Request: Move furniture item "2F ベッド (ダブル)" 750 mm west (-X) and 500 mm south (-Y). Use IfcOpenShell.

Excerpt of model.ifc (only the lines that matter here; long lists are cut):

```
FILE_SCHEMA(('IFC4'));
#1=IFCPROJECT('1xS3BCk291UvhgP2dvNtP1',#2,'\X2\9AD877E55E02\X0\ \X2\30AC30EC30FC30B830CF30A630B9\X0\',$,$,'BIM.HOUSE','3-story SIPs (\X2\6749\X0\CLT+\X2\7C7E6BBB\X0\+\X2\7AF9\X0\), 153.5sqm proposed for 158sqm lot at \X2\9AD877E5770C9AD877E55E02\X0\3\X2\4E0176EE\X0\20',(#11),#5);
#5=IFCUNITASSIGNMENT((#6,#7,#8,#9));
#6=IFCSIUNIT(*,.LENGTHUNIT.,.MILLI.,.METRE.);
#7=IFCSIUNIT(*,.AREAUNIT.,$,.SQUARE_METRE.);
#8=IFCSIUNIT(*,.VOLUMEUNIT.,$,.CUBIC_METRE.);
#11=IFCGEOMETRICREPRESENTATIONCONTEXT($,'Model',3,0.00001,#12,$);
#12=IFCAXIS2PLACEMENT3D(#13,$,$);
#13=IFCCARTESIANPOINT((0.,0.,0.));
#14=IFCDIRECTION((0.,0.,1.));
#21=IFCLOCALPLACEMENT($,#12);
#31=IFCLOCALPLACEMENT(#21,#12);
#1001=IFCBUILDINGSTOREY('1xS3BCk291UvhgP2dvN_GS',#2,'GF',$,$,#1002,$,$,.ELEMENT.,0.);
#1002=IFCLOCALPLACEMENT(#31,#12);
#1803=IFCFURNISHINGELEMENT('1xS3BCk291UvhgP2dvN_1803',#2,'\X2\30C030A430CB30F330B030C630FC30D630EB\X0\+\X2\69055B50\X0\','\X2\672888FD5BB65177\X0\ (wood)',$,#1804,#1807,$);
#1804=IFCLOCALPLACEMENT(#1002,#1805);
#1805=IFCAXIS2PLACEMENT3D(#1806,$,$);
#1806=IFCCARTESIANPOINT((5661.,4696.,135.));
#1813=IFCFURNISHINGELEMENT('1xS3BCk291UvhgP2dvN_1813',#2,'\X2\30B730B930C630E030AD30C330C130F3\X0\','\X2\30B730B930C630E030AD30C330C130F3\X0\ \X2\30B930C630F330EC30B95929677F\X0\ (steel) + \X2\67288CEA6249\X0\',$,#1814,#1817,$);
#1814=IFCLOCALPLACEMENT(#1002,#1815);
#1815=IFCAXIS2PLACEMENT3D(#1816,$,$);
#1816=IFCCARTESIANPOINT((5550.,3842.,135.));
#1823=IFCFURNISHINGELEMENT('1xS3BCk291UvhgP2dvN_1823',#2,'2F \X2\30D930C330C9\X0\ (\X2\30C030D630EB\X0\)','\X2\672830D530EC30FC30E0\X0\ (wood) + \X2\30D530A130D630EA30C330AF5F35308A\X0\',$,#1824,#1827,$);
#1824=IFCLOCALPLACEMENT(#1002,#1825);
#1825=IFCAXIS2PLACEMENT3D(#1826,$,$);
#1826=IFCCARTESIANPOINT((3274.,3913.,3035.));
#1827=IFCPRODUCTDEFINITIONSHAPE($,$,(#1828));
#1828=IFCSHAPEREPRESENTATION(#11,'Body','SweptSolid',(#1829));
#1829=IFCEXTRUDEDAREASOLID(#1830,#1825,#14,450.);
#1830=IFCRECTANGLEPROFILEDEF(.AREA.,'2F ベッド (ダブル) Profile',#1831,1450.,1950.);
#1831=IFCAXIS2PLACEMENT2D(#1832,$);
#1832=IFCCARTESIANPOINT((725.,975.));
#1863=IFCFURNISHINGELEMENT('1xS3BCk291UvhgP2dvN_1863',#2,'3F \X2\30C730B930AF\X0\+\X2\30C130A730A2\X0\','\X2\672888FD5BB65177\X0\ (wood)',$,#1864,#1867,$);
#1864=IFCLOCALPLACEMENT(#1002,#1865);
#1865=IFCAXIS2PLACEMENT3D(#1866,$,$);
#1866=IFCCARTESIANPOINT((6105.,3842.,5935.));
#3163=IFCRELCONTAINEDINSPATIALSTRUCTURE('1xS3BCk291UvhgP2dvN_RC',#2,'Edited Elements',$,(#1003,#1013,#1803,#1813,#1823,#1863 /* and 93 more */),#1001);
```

```python
import ifcopenshell
import ifcopenshell.api.geometry
import ifcopenshell.util.placement
import ifcopenshell.util.unit

model = ifcopenshell.open("model.ifc")
unit_scale = ifcopenshell.util.unit.calculate_unit_scale(model)

item = model.by_guid("1xS3BCk291UvhgP2dvN_1823")
matrix = ifcopenshell.util.placement.get_local_placement(item.ObjectPlacement)
matrix[0, 3] -= 0.75 / unit_scale
matrix[1, 3] -= 0.5 / unit_scale
ifcopenshell.api.geometry.edit_object_placement(model, product=item, matrix=matrix, is_si=False)

print(ifcopenshell.util.placement.get_local_placement(item.ObjectPlacement).round(3) + 0.0)

model.write("model_updated.ifc")
```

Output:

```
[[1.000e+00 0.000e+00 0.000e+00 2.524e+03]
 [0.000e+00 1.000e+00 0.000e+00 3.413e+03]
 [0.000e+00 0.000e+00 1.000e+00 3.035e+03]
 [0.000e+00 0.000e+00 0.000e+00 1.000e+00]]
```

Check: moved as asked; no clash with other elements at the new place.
